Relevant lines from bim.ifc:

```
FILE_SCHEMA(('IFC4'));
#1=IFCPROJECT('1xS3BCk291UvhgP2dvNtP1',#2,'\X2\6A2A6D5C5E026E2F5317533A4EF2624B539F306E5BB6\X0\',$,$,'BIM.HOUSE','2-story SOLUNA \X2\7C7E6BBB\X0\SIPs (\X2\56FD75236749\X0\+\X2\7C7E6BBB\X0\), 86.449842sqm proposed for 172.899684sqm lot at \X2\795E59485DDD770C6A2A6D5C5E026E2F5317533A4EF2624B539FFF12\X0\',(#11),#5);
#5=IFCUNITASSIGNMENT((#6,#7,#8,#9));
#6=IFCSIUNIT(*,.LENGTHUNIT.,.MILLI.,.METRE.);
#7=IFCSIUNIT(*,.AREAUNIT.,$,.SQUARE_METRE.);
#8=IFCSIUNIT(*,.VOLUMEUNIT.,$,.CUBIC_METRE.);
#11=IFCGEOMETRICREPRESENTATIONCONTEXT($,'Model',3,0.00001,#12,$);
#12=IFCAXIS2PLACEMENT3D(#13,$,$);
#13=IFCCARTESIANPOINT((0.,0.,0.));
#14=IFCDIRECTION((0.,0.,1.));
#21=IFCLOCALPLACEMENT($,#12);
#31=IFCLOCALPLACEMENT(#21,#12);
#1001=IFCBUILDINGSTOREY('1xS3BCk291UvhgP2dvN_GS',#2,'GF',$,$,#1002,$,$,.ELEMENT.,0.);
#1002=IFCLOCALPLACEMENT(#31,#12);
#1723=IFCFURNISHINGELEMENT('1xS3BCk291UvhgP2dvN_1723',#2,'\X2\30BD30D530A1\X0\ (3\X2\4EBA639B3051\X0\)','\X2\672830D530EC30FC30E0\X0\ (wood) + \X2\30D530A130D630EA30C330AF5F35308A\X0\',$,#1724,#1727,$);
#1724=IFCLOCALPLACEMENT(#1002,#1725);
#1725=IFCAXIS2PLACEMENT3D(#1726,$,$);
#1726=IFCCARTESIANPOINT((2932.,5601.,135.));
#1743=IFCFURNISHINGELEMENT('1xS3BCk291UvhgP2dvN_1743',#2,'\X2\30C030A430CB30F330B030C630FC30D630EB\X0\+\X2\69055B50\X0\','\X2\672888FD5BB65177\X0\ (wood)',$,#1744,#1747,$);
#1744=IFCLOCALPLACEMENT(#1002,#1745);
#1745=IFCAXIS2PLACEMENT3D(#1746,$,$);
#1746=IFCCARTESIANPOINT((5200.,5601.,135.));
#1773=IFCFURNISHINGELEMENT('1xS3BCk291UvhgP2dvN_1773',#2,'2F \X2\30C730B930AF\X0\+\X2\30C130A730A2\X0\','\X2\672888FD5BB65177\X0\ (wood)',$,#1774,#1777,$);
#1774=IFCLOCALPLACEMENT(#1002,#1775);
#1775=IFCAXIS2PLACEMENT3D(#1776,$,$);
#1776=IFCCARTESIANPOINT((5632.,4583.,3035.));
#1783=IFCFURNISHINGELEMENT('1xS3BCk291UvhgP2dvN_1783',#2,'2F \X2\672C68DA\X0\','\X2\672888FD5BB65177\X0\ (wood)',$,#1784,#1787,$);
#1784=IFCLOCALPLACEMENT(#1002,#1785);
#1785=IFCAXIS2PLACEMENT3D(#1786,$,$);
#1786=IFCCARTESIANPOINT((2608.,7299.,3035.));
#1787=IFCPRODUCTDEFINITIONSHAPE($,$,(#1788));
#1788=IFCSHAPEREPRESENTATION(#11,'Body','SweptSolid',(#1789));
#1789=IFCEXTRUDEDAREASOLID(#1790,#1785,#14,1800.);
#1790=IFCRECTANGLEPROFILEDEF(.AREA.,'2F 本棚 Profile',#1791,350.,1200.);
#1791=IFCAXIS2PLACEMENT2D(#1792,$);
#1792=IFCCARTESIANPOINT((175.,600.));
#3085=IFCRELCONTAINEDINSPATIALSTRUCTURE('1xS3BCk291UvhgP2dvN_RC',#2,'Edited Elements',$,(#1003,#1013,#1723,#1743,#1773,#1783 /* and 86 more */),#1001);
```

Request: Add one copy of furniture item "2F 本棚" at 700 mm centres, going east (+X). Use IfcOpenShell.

```python
import numpy as np
import ifcopenshell
import ifcopenshell.api.geometry
import ifcopenshell.api.root
import ifcopenshell.util.element
import ifcopenshell.util.placement

model = ifcopenshell.open("bim.ifc")


def reuse_history(source, copy):
    """copy_class also copies each property set's owner history, people and application; keep the originals."""
    for rel in copy.IsDefinedBy:
        if rel.is_a("IfcRelDefinesByProperties") and (history := rel.RelatingPropertyDefinition.OwnerHistory):
            rel.RelatingPropertyDefinition.OwnerHistory = source.OwnerHistory
            ifcopenshell.util.element.remove_deep2(model, history)


source = model.by_id(1783)
base = ifcopenshell.util.placement.get_local_placement(source.ObjectPlacement)
step = np.array([1.0, 0.0, 0.0]) * 700.0

for i in range(1, 2):
    copy = ifcopenshell.api.root.copy_class(model, product=source)
    copy.Representation = ifcopenshell.util.element.copy_deep(
        model, source.Representation, exclude=["IfcGeometricRepresentationContext", "IfcRepresentationMap"]
    )
    reuse_history(source, copy)
    matrix = base.copy()
    matrix[:3, 3] += i * step
    print("added at", matrix[:3, 3].round(3) + 0.0)
    ifcopenshell.api.geometry.edit_object_placement(model, product=copy, matrix=matrix, is_si=False)

model.write("bim-out.ifc")
```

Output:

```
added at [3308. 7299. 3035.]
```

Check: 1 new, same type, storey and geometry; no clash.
